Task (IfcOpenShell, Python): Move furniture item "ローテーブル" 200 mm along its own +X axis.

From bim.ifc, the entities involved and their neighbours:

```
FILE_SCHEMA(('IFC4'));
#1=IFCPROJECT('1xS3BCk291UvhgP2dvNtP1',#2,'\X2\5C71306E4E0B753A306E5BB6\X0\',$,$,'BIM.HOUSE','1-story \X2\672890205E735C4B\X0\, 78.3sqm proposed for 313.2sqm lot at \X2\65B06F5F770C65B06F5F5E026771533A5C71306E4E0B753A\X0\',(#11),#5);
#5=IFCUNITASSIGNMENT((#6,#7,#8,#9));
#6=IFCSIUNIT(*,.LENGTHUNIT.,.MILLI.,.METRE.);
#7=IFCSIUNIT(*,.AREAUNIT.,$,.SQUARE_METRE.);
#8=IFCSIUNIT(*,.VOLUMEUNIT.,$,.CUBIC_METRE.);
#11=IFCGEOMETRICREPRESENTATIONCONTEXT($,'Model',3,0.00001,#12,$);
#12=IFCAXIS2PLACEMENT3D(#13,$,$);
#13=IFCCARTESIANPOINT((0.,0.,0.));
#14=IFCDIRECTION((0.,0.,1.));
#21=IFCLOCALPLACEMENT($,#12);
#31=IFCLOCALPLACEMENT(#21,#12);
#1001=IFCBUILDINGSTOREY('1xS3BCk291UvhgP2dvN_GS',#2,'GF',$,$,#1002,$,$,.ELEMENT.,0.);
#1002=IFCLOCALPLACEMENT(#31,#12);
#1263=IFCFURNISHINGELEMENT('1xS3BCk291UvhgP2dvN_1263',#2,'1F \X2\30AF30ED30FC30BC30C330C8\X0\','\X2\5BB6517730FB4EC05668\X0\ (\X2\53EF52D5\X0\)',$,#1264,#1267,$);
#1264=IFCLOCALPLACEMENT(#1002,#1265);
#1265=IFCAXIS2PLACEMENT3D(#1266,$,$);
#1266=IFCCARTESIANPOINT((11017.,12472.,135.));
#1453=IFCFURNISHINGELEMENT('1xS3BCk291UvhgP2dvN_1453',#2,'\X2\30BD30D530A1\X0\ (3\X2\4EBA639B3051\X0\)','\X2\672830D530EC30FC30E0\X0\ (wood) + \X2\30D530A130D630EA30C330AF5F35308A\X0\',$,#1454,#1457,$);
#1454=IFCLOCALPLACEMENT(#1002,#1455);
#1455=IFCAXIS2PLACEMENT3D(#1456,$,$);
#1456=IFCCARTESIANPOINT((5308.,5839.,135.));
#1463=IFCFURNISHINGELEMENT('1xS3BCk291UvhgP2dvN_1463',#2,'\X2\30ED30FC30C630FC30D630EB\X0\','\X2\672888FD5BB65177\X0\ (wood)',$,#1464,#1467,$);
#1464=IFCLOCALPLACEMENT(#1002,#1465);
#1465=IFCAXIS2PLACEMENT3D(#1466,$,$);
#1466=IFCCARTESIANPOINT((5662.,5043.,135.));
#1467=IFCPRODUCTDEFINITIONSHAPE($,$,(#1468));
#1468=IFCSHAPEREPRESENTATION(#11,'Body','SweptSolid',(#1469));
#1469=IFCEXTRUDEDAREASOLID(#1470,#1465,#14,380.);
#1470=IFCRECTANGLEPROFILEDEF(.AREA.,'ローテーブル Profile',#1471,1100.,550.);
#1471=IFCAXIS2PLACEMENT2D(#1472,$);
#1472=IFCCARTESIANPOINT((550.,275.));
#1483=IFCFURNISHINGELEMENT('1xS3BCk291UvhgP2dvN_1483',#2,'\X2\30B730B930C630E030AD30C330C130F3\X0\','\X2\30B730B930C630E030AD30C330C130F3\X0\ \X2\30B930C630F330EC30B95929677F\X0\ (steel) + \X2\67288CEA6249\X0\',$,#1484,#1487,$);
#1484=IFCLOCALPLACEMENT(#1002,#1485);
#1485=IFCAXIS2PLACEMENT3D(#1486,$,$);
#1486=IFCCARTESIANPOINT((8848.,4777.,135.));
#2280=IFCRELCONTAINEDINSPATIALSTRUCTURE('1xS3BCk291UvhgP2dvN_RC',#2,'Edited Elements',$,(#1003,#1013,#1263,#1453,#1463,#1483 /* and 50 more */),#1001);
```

```python
import ifcopenshell
import ifcopenshell.api.geometry
import ifcopenshell.util.placement
import ifcopenshell.util.unit

model = ifcopenshell.open("bim.ifc")
unit_scale = ifcopenshell.util.unit.calculate_unit_scale(model)

item = model.by_id(1463)
matrix = ifcopenshell.util.placement.get_local_placement(item.ObjectPlacement)
matrix[:3, 3] += matrix[:3, 0] * 0.2 / unit_scale
ifcopenshell.api.geometry.edit_object_placement(model, product=item, matrix=matrix, is_si=False)

print(ifcopenshell.util.placement.get_local_placement(item.ObjectPlacement).round(3) + 0.0)

model.write("bim_updated.ifc")
```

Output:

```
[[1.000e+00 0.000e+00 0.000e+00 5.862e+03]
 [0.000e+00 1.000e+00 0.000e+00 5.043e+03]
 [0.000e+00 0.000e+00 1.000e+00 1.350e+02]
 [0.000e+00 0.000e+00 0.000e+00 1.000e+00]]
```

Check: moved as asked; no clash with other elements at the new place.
